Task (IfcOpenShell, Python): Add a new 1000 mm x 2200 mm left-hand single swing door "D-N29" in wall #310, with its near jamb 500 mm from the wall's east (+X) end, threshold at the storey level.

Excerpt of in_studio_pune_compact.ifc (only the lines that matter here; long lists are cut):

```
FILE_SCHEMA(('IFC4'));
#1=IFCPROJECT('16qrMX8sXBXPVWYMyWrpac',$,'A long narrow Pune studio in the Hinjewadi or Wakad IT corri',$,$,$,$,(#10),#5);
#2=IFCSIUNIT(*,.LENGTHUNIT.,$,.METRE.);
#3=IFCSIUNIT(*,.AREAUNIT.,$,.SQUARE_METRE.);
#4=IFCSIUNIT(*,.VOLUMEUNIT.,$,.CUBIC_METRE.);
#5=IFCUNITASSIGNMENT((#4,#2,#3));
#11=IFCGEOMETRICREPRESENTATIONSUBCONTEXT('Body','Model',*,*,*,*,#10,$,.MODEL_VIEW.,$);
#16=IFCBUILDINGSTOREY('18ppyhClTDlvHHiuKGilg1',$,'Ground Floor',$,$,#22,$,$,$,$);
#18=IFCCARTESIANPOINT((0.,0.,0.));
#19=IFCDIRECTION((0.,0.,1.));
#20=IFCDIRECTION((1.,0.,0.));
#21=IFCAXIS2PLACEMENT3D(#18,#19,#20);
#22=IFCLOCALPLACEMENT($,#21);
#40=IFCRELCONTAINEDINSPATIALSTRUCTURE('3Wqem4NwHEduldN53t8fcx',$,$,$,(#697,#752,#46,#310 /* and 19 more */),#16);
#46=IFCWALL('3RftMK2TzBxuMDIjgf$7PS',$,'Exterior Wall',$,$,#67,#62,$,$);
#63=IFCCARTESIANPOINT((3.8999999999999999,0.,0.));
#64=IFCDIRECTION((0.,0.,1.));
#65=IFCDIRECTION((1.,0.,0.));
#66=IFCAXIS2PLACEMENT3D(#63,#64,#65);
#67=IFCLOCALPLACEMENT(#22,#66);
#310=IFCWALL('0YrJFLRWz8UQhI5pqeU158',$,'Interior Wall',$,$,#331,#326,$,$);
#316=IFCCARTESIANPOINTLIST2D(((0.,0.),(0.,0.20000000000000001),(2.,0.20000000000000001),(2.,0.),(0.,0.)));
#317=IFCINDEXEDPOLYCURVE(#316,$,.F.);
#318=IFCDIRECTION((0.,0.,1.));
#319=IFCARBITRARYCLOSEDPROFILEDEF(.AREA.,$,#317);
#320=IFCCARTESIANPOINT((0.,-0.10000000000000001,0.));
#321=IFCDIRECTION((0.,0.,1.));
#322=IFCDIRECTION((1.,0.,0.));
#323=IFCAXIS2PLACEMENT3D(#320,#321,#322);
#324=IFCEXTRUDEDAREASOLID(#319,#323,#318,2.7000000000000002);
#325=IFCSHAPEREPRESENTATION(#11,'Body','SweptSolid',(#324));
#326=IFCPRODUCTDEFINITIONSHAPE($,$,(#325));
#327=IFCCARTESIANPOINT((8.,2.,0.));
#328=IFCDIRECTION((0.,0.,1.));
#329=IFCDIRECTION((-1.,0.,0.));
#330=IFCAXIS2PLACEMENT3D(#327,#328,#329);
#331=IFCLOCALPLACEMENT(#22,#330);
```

```python
import numpy as np
import ifcopenshell
import ifcopenshell.api.feature
import ifcopenshell.api.geometry
import ifcopenshell.api.root
import ifcopenshell.api.spatial
import ifcopenshell.geom
import ifcopenshell.util.element
import ifcopenshell.util.placement
import ifcopenshell.util.representation
import ifcopenshell.util.shape
import ifcopenshell.util.unit

model = ifcopenshell.open("in_studio_pune_compact.ifc")
unit_scale = ifcopenshell.util.unit.calculate_unit_scale(model)
settings = ifcopenshell.geom.settings()


def volume(element):
    """Net volume in cubic metres, openings subtracted."""
    shape = ifcopenshell.geom.create_shape(settings, element)
    return ifcopenshell.util.shape.get_volume(shape.geometry)


wall = model.by_id(310)
storey = ifcopenshell.util.element.get_container(wall, ifc_class="IfcBuildingStorey")
context = ifcopenshell.util.representation.get_context(model, "Model", "Body", "MODEL_VIEW")
before = volume(wall)

width, height, from_end, sill = 1, 2.2, 0.5, 0.0  # metres

# The wall runs along its own X axis, and the end named is its -X end.
wall_shape = ifcopenshell.geom.create_shape(settings, wall)
x, y, z = ifcopenshell.util.shape.get_vertices(wall_shape.geometry).T
start = x.min() + from_end
face, thickness = float(y.min()), float(y.max() - y.min())
wall_matrix = ifcopenshell.util.placement.get_local_placement(wall.ObjectPlacement)
level = ifcopenshell.util.placement.get_local_placement(storey.ObjectPlacement)[2, 3]


def in_wall(x, y):
    """Placement at x, y metres in the wall's axes, at sill height."""
    matrix = wall_matrix.copy()
    matrix[:, 3] = wall_matrix @ np.array([x / unit_scale, y / unit_scale, 0.0, 1.0])
    matrix[2, 3] = level + sill / unit_scale
    return matrix


# Opening: a box that overshoots both wall faces by 50 mm.
opening = ifcopenshell.api.root.create_entity(model, ifc_class="IfcOpeningElement", predefined_type="OPENING")
box = ifcopenshell.api.geometry.add_wall_representation(
    model, context=context, length=width, height=height, thickness=thickness + 0.1
)
ifcopenshell.api.geometry.assign_representation(model, product=opening, representation=box)
ifcopenshell.api.geometry.edit_object_placement(model, product=opening, matrix=in_wall(start, face - 0.05), is_si=False)
ifcopenshell.api.feature.add_feature(model, feature=opening, element=wall)

door = ifcopenshell.api.root.create_entity(model, ifc_class="IfcDoor", name="D-N29", predefined_type="DOOR")
door.OverallWidth, door.OverallHeight = width / unit_scale, height / unit_scale
door.OperationType = "SINGLE_SWING_LEFT"
body = ifcopenshell.api.geometry.add_door_representation(
    model,
    context=context,
    overall_width=door.OverallWidth,
    overall_height=door.OverallHeight,
    operation_type="SINGLE_SWING_LEFT",
    lining_properties={"LiningDepth": thickness / unit_scale, "ThresholdDepth": thickness / unit_scale},
)
ifcopenshell.api.geometry.assign_representation(model, product=door, representation=body)
ifcopenshell.api.spatial.assign_container(model, products=[door], relating_structure=storey)
ifcopenshell.api.feature.add_filling(model, opening=opening, element=door)

# The lining spans the wall, so the door starts at the wall face.
ifcopenshell.api.geometry.edit_object_placement(model, product=door, matrix=in_wall(start, face), is_si=False)

after = volume(wall)

print(f"wall volume {before:.3f} -> {after:.3f} m3")

model.write("in_studio_pune_compact_rev.ifc")
```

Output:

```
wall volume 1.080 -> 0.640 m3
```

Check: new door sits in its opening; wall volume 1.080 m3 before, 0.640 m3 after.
